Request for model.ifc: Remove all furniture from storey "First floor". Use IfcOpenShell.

First a look at what the model holds.

```python
import ifcopenshell
import ifcopenshell.util.element

model = ifcopenshell.open("model.ifc")
print(model.schema)
storey = next(s for s in model.by_type("IfcBuildingStorey") if s.Name == "First floor")
furniture = [e for e in ifcopenshell.util.element.get_decomposition(storey) if e.is_a("IfcFurnishingElement")]
seen = {}
for e in furniture:
    element_type = ifcopenshell.util.element.get_type(e)
    name = element_type.Name if element_type not in (None, e) else None
    seen[name] = seen.get(name, 0) + 1
for name, count in sorted(seen.items(), key=str):
    print(count, "x", name)
```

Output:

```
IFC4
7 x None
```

```python
import ifcopenshell
import ifcopenshell.api.root
import ifcopenshell.util.element

model = ifcopenshell.open("model.ifc")

storey = next(s for s in model.by_type("IfcBuildingStorey") if s.Name == "First floor")
furniture = [e for e in ifcopenshell.util.element.get_decomposition(storey) if e.is_a("IfcFurnishingElement")]

for e in furniture:
    ifcopenshell.api.root.remove_product(model, product=e)
print(len(furniture), "removed")

model.write("model_edited.ifc")
```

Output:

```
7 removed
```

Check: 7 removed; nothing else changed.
